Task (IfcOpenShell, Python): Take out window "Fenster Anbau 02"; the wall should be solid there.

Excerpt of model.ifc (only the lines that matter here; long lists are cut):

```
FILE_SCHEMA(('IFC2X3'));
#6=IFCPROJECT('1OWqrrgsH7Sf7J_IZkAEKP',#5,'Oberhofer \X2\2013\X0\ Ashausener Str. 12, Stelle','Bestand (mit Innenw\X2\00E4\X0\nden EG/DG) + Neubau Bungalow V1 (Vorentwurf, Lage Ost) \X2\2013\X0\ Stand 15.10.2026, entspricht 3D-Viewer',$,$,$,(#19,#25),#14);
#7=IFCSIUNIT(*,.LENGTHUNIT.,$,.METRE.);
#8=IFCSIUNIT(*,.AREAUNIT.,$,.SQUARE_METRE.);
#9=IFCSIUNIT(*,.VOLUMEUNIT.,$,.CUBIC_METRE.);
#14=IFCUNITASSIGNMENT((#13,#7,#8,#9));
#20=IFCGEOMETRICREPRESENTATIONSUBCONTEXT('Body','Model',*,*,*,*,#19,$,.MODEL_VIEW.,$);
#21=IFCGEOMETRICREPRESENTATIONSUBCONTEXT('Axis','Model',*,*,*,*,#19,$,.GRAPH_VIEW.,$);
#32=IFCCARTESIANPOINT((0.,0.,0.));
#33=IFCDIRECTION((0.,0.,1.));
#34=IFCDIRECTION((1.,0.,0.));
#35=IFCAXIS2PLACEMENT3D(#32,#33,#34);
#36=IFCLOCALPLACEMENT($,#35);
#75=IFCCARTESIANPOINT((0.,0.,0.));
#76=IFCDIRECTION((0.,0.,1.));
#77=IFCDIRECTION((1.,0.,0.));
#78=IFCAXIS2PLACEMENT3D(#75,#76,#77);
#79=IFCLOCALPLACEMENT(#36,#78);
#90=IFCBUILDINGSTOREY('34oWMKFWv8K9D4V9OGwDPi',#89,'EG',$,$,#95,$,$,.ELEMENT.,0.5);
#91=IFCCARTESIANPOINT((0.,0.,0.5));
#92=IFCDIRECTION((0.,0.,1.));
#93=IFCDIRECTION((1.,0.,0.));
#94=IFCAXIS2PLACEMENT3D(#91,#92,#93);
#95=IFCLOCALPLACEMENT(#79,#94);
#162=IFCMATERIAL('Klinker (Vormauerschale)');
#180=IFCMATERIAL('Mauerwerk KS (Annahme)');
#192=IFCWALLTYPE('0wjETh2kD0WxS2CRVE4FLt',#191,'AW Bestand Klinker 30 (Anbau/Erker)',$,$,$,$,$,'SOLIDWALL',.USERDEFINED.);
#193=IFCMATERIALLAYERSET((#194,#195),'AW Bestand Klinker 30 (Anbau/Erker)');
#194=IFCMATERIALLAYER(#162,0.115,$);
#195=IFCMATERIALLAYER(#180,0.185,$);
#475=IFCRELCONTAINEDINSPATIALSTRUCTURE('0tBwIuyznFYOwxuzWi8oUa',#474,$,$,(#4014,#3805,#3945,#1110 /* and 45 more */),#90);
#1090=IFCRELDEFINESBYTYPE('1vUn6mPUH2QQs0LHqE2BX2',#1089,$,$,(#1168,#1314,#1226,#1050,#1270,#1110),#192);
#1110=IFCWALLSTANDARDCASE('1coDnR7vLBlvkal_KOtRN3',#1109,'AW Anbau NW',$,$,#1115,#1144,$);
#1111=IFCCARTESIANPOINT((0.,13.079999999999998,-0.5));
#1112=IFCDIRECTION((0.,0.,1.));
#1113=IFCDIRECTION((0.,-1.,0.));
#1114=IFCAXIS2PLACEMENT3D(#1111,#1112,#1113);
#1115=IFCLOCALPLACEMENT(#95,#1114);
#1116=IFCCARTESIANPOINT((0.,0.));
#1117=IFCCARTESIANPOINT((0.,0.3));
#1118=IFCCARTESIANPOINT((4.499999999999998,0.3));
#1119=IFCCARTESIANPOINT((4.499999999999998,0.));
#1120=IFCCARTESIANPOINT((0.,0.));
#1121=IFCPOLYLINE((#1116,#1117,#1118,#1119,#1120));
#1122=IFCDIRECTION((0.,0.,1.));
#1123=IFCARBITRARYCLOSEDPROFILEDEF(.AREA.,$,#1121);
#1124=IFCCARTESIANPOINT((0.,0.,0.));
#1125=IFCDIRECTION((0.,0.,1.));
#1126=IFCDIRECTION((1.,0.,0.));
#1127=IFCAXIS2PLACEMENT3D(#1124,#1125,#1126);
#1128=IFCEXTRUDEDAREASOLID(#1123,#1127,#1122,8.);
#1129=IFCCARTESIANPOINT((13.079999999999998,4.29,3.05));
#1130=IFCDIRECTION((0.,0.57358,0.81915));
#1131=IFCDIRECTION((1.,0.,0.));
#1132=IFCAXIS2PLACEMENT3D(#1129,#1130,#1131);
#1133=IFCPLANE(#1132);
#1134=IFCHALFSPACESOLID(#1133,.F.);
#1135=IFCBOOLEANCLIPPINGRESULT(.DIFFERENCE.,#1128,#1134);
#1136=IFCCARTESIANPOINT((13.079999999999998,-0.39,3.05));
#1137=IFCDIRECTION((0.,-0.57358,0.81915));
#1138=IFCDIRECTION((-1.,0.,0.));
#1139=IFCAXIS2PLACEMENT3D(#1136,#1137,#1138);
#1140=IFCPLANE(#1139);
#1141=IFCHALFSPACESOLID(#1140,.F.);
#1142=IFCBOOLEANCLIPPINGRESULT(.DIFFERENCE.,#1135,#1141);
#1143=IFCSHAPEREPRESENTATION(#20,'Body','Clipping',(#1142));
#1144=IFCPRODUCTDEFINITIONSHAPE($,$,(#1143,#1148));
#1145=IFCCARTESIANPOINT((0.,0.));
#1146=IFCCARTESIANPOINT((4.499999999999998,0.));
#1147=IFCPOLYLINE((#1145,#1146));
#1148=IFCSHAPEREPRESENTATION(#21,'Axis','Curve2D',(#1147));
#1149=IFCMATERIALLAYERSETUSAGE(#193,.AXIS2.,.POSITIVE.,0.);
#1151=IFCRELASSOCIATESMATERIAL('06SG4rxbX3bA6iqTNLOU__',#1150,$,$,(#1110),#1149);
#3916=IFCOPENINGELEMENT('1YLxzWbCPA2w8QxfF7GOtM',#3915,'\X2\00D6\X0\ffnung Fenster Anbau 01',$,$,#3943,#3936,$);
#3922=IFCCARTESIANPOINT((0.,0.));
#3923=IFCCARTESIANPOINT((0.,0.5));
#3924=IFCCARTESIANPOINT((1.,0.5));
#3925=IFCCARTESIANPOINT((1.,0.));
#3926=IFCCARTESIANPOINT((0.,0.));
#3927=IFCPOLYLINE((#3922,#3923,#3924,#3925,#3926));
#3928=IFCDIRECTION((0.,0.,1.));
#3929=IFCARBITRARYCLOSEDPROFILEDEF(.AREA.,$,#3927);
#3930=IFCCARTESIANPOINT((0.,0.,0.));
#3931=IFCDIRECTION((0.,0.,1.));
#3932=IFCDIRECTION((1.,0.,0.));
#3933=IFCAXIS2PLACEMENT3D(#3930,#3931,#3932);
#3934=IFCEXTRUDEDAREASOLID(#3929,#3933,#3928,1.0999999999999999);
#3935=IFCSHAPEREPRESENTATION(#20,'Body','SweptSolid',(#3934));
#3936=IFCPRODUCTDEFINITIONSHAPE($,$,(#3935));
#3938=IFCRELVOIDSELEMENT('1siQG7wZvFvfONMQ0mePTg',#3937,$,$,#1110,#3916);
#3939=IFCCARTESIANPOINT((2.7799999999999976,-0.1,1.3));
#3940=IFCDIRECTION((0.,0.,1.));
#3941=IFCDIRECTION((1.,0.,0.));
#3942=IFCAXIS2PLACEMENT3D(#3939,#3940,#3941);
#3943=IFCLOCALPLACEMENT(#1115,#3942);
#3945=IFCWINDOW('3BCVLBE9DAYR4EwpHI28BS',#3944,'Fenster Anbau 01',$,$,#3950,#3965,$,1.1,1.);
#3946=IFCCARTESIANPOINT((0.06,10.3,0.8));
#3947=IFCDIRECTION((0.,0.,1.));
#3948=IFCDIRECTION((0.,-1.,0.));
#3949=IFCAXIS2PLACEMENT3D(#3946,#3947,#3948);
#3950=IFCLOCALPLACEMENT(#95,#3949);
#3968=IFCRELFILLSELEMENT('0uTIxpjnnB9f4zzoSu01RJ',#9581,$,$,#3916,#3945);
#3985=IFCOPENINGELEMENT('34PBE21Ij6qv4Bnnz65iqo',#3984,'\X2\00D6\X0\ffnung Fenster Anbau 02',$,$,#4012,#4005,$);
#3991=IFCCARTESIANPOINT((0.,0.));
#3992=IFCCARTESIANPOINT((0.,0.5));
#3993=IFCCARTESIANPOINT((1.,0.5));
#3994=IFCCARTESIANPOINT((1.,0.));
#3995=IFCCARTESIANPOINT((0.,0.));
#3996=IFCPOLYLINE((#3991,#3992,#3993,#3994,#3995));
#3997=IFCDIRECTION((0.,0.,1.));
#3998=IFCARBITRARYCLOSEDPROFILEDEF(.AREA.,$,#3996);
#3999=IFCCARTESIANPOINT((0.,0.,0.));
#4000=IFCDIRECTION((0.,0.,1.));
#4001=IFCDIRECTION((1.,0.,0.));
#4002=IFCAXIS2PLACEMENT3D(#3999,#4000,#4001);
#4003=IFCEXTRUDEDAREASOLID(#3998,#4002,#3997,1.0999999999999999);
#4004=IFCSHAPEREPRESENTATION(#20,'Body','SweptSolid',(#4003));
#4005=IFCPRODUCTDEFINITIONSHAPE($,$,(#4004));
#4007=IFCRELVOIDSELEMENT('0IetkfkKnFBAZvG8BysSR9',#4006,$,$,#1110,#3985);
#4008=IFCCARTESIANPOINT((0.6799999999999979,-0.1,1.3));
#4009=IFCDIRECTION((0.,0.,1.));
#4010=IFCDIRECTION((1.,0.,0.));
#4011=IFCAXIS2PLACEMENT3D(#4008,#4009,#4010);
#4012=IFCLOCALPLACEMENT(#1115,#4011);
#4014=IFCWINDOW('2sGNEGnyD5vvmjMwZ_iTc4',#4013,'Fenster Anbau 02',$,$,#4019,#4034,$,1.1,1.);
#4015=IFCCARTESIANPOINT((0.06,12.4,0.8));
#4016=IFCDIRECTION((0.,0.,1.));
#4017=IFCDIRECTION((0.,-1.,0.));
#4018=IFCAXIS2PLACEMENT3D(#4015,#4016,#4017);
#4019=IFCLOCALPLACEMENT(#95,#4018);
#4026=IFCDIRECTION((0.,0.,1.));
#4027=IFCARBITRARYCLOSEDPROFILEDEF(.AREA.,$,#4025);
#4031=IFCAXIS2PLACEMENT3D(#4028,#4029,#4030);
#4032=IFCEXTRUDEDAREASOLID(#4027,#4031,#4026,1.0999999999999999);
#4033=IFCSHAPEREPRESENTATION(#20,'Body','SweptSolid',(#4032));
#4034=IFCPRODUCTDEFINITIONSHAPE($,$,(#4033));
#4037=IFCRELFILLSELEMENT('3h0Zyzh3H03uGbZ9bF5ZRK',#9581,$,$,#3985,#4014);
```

```python
import ifcopenshell
import ifcopenshell.api.feature
import ifcopenshell.api.root
import ifcopenshell.geom
import ifcopenshell.util.shape

model = ifcopenshell.open("model.ifc")
settings = ifcopenshell.geom.settings()


def volume(element):
    """Net volume in cubic metres, openings subtracted."""
    shape = ifcopenshell.geom.create_shape(settings, element)
    return ifcopenshell.util.shape.get_volume(shape.geometry)


window = model.by_guid("2sGNEGnyD5vvmjMwZ_iTc4")
opening = window.FillsVoids[0].RelatingOpeningElement
wall = opening.VoidsElements[0].RelatingBuildingElement
before = volume(wall)

ifcopenshell.api.root.remove_product(model, product=window)
ifcopenshell.api.feature.remove_feature(model, feature=opening)

after = volume(wall)

print(f"wall volume {before:.3f} -> {after:.3f} m3")

model.write("model_rev.ifc")
```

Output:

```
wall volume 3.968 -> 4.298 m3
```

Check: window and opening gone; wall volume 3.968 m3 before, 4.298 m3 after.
